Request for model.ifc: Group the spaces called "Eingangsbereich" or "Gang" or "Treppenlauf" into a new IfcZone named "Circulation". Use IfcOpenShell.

First a look at what the model holds.

```python
import ifcopenshell

model = ifcopenshell.open("model.ifc")
print(model.schema)
seen = {}
for space in model.by_type("IfcSpace"):
    seen[space.LongName] = seen.get(space.LongName, 0) + 1
for name, count in sorted(seen.items(), key=str):
    print(count, "x", name)
print("zones:", [z.Name for z in model.by_type("IfcZone")][:20])
```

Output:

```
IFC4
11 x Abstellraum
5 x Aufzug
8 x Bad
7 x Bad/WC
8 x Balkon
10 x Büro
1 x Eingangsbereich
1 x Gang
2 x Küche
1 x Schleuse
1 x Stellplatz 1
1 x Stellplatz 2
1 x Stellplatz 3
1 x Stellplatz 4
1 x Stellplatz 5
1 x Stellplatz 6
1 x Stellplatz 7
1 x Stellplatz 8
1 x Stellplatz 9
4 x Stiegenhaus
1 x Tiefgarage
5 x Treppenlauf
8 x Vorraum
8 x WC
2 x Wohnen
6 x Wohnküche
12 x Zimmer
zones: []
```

```python
import ifcopenshell
import ifcopenshell.api.group
import ifcopenshell.api.root

model = ifcopenshell.open("model.ifc")

names = {"Eingangsbereich", "Gang", "Treppenlauf"}
spaces = [s for s in model.by_type("IfcSpace") if s.LongName in names]

zone = ifcopenshell.api.root.create_entity(model, ifc_class="IfcZone", name="Circulation")
ifcopenshell.api.group.assign_group(model, products=spaces, group=zone)
print(len(spaces), "spaces in", zone.Name)

model.write("model_edited.ifc")
```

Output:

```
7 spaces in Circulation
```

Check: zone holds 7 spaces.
